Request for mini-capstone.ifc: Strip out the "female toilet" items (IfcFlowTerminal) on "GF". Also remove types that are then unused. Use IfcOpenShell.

First a look at what the model holds.

```python
import ifcopenshell
import ifcopenshell.util.element

model = ifcopenshell.open("mini-capstone.ifc")
print(model.schema)
storey = next(s for s in model.by_type("IfcBuildingStorey") if s.Name == "GF")
terminals = [e for e in ifcopenshell.util.element.get_decomposition(storey) if e.is_a("IfcFlowTerminal")]
seen = {}
for e in terminals:
    element_type = ifcopenshell.util.element.get_type(e)
    name = element_type.Name if element_type not in (None, e) else None
    seen[name] = seen.get(name, 0) + 1
for name, count in sorted(seen.items(), key=str):
    print(count, "x", name)
```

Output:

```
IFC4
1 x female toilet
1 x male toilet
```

```python
import ifcopenshell
import ifcopenshell.api.root
import ifcopenshell.util.element

model = ifcopenshell.open("mini-capstone.ifc")

storey = next(s for s in model.by_type("IfcBuildingStorey") if s.Name == "GF")
terminals = [e for e in ifcopenshell.util.element.get_decomposition(storey) if e.is_a("IfcFlowTerminal")]
targets = [e for e in terminals if (t := ifcopenshell.util.element.get_type(e)) not in (None, e) and t.Name == "female toilet"]
types = {ifcopenshell.util.element.get_type(e) for e in targets} - {None, *targets}

for e in targets:
    ifcopenshell.api.root.remove_product(model, product=e)
print(len(targets), "removed")

unused = [t for t in types if not ifcopenshell.util.element.get_types(t)]
for t in unused:
    ifcopenshell.api.root.remove_product(model, product=t)
print(len(unused), "unused types removed")

model.write("mini-capstone_updated.ifc")
```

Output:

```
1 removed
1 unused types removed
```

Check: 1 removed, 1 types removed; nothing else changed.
